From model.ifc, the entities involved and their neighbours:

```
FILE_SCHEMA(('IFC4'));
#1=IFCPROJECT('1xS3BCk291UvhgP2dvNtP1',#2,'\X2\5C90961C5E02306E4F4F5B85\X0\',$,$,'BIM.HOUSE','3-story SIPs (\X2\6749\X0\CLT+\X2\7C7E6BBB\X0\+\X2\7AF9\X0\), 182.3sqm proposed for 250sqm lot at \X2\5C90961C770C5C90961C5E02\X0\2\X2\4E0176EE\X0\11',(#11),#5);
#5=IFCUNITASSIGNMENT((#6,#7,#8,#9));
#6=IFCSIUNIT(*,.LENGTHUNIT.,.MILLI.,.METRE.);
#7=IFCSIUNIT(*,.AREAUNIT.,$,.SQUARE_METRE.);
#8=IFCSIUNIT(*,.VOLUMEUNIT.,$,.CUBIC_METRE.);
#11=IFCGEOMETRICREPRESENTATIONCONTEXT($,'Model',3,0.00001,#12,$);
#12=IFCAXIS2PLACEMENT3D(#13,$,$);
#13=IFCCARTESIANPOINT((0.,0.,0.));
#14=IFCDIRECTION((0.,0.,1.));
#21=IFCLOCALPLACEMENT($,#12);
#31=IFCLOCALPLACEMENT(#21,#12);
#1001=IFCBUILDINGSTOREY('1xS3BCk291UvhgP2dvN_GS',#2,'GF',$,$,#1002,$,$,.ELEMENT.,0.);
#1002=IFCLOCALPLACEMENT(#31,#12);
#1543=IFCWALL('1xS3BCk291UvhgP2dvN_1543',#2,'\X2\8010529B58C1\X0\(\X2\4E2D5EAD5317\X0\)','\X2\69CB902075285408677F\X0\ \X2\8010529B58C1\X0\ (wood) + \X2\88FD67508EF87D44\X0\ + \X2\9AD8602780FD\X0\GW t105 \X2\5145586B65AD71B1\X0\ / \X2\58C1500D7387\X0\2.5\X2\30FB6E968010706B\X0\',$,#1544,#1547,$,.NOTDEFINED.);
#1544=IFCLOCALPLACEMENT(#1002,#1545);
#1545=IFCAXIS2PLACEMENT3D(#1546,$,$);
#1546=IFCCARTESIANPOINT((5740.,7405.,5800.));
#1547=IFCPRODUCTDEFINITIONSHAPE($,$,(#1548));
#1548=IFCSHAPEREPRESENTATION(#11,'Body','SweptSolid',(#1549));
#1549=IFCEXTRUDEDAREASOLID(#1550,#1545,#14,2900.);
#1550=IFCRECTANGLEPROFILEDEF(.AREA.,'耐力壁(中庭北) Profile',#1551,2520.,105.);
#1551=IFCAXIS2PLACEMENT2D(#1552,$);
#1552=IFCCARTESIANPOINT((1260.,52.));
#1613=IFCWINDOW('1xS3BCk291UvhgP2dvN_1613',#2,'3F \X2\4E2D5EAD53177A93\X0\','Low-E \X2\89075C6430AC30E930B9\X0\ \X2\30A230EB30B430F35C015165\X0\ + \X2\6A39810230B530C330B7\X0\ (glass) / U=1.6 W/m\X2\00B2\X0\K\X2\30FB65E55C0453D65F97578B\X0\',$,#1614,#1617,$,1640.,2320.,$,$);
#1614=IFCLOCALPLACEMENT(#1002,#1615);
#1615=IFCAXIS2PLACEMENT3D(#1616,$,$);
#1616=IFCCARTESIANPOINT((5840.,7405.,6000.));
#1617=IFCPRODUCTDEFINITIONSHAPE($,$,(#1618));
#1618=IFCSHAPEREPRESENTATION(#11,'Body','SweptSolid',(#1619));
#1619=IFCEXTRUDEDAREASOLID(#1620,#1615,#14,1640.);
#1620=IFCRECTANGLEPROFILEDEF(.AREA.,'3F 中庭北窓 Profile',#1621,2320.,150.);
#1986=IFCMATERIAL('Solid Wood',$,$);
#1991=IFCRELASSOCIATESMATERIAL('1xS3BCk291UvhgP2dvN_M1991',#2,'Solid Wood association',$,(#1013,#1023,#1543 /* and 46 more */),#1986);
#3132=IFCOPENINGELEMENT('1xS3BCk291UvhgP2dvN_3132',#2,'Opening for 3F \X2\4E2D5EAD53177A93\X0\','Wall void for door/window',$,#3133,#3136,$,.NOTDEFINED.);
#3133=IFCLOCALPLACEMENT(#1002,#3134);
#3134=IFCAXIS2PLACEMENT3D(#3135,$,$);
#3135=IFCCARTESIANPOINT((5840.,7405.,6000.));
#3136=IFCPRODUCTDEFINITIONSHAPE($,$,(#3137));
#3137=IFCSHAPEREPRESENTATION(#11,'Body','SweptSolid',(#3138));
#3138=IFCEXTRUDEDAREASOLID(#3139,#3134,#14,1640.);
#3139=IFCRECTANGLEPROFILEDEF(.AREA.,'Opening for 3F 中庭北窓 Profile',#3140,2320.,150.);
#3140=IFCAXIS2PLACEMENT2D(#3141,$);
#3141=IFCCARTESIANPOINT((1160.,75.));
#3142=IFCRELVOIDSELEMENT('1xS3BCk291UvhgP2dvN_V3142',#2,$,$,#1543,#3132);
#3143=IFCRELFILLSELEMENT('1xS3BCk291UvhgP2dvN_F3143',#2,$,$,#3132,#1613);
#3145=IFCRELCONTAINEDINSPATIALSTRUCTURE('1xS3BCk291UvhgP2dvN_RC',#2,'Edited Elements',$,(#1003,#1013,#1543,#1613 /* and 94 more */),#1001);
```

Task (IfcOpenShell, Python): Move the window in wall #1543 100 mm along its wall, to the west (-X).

```python
import ifcopenshell
import ifcopenshell.api.geometry
import ifcopenshell.util.placement
import ifcopenshell.util.unit

model = ifcopenshell.open("model.ifc")
unit_scale = ifcopenshell.util.unit.calculate_unit_scale(model)

window = model.by_guid("1xS3BCk291UvhgP2dvN_1613")
opening = window.FillsVoids[0].RelatingOpeningElement
wall = opening.VoidsElements[0].RelatingBuildingElement

wall_matrix = ifcopenshell.util.placement.get_local_placement(wall.ObjectPlacement)
shift = wall_matrix[:3, 0] * -0.1 / unit_scale
before = ifcopenshell.util.placement.get_local_placement(window.ObjectPlacement)[:3, 3].copy()

# The window is not placed relative to its opening, so move both.
for product in (opening, window):
    matrix = ifcopenshell.util.placement.get_local_placement(product.ObjectPlacement)
    matrix[:3, 3] += shift
    ifcopenshell.api.geometry.edit_object_placement(model, product=product, matrix=matrix, is_si=False)

after = ifcopenshell.util.placement.get_local_placement(window.ObjectPlacement)[:3, 3]
print("window moved by", (after - before).round(3) + 0.0)

model.write("model-out.ifc")
```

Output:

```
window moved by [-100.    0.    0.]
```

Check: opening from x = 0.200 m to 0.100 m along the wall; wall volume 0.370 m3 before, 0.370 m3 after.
